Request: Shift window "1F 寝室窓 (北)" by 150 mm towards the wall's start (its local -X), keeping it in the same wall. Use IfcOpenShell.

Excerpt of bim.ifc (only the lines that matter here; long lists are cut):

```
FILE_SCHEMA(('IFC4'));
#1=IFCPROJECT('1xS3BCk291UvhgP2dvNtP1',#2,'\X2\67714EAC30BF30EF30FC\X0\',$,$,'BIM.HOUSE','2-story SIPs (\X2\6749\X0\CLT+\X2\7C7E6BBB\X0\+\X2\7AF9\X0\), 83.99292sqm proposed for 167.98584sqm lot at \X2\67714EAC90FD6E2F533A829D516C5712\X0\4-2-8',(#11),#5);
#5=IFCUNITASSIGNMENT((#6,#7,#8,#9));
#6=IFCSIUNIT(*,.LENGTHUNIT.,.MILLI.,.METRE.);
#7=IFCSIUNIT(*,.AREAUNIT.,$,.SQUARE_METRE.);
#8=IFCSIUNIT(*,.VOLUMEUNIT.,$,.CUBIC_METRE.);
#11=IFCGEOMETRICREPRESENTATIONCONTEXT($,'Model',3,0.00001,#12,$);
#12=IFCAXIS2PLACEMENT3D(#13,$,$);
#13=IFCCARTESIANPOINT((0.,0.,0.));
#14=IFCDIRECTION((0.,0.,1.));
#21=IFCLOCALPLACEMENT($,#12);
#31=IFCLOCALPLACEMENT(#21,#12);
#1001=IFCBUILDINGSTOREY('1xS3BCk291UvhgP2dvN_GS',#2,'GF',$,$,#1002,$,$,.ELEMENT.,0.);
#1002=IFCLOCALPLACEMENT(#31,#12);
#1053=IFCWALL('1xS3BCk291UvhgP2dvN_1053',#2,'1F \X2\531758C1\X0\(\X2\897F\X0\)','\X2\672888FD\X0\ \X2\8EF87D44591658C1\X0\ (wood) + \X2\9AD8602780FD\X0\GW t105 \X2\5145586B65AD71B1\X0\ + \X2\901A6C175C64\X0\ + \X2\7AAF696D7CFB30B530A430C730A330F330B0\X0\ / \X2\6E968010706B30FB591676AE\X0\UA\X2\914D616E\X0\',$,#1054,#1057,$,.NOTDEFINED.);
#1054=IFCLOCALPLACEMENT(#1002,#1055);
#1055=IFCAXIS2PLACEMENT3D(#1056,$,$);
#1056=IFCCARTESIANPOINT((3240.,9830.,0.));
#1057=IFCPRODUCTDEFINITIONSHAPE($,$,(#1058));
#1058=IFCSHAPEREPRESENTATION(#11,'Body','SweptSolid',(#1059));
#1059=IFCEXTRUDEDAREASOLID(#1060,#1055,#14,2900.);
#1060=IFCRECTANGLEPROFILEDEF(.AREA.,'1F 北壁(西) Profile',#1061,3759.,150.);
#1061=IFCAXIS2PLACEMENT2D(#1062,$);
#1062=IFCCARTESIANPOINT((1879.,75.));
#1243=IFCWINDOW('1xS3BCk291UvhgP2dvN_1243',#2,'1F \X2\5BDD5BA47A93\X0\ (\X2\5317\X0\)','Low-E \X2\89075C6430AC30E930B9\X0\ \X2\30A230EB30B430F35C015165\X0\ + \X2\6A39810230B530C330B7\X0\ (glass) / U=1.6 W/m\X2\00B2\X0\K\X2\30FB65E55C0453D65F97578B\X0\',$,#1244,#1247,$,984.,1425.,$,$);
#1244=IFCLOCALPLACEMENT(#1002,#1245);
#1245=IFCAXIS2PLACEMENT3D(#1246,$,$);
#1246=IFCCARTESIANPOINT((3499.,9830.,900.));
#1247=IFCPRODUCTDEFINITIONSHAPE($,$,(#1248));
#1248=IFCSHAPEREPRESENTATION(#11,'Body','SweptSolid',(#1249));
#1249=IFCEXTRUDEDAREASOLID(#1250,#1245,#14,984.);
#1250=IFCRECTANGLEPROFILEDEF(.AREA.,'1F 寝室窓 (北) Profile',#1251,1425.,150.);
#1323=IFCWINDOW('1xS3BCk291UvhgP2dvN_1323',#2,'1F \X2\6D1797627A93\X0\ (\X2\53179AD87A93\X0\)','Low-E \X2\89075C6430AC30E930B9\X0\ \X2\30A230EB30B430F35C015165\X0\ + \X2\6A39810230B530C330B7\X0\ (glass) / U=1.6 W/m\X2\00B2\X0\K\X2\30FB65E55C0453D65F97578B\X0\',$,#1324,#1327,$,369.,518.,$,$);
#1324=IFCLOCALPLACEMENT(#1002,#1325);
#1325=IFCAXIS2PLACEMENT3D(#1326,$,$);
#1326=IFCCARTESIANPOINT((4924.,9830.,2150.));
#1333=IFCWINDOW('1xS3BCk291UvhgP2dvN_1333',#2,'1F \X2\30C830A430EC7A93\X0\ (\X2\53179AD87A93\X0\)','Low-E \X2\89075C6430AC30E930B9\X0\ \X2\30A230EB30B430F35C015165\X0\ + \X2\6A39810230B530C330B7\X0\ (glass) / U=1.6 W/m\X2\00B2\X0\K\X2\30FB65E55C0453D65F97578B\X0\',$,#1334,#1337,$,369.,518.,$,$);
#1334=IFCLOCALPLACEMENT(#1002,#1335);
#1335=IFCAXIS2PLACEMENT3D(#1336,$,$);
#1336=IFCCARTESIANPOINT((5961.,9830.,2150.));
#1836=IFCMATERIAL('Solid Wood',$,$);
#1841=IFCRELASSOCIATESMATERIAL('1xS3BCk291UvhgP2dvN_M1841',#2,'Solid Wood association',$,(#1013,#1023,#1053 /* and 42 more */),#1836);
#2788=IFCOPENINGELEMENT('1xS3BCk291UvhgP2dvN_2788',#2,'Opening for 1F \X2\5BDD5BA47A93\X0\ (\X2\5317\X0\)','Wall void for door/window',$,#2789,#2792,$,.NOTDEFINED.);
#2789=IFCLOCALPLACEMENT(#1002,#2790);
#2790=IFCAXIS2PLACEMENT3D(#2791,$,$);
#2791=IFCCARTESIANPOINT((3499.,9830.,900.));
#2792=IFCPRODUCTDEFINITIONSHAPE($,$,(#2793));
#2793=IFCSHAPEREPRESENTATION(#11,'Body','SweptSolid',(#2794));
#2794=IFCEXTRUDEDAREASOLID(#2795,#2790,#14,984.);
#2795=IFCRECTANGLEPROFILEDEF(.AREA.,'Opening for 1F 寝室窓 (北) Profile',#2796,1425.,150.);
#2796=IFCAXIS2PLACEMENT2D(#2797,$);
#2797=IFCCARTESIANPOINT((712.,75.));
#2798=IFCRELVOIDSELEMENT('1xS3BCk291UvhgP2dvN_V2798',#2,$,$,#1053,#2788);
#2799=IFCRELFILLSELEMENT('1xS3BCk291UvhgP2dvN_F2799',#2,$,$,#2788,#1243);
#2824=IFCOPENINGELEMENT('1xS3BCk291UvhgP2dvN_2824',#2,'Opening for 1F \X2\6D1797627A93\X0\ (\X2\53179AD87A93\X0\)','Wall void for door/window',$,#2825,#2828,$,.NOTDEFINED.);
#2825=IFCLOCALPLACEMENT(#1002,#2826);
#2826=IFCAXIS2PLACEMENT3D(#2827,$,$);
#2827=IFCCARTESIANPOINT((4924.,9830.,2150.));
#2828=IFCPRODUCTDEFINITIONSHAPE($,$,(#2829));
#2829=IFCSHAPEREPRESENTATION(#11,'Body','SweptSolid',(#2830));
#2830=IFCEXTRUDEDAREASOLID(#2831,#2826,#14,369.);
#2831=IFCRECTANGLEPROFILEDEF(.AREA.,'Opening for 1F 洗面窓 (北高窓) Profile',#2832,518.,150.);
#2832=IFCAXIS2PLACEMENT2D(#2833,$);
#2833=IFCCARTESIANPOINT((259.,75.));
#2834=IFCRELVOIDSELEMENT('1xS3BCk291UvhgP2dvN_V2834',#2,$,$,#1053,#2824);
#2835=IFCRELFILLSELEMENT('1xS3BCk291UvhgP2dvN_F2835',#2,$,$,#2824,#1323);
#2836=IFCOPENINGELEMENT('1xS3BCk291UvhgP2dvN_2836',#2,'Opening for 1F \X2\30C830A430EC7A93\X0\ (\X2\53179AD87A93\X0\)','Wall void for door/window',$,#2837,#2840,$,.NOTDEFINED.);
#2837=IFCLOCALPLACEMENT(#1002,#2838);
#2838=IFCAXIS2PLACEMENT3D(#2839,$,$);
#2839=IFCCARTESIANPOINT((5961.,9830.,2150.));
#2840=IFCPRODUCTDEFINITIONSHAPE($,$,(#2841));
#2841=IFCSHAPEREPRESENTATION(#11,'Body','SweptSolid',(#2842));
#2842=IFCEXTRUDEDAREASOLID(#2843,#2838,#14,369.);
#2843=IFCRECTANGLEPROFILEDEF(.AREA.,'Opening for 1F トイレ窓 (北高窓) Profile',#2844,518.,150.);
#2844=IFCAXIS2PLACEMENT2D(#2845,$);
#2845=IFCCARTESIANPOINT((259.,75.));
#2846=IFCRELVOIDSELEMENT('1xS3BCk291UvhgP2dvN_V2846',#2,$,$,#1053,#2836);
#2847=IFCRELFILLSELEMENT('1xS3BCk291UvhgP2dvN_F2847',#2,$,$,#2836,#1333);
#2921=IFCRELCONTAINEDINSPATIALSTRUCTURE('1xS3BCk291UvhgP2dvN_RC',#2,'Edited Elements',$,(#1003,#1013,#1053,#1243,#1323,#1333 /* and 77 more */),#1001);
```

```python
import ifcopenshell
import ifcopenshell.api.geometry
import ifcopenshell.util.placement
import ifcopenshell.util.unit

model = ifcopenshell.open("bim.ifc")
unit_scale = ifcopenshell.util.unit.calculate_unit_scale(model)

window = model.by_guid("1xS3BCk291UvhgP2dvN_1243")
opening = window.FillsVoids[0].RelatingOpeningElement
wall = opening.VoidsElements[0].RelatingBuildingElement

wall_matrix = ifcopenshell.util.placement.get_local_placement(wall.ObjectPlacement)
shift = wall_matrix[:3, 0] * -0.15 / unit_scale
before = ifcopenshell.util.placement.get_local_placement(window.ObjectPlacement)[:3, 3].copy()

# The window is not placed relative to its opening, so move both.
for product in (opening, window):
    matrix = ifcopenshell.util.placement.get_local_placement(product.ObjectPlacement)
    matrix[:3, 3] += shift
    ifcopenshell.api.geometry.edit_object_placement(model, product=product, matrix=matrix, is_si=False)

after = ifcopenshell.util.placement.get_local_placement(window.ObjectPlacement)[:3, 3]
print("window moved by", (after - before).round(3) + 0.0)

model.write("bim_v2.ifc")
```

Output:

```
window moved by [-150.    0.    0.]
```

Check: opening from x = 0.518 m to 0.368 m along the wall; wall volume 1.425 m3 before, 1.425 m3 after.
